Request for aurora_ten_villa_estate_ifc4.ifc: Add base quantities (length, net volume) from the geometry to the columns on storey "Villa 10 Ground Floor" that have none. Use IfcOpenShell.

First a look at what the model holds.

```python
import ifcopenshell
import ifcopenshell.util.element
import ifcopenshell.util.unit

model = ifcopenshell.open("aurora_ten_villa_estate_ifc4.ifc")
print(model.schema)
for unit_type in ("LENGTHUNIT", "AREAUNIT", "VOLUMEUNIT"):
    print(unit_type, ifcopenshell.util.unit.calculate_unit_scale(model, unit_type))
storey = next(s for s in model.by_type("IfcBuildingStorey") if s.Name == "Villa 10 Ground Floor")
columns = [e for e in ifcopenshell.util.element.get_decomposition(storey) if e.is_a("IfcColumn")]
for e in sorted(columns, key=lambda e: e.id()):
    print(e.id(), e.is_a(), e.Name, list(ifcopenshell.util.element.get_psets(e, qtos_only=True)), sep=" | ")
```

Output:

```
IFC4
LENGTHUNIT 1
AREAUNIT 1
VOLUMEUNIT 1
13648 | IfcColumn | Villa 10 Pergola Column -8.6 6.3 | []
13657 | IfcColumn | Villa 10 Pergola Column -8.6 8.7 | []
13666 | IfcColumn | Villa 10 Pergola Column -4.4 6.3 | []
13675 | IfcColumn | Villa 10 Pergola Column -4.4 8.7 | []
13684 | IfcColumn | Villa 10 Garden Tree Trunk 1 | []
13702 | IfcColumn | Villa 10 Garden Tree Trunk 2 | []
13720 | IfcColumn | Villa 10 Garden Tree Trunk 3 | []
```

```python
import ifcopenshell
import ifcopenshell.api.pset
import ifcopenshell.geom
import ifcopenshell.util.element
import ifcopenshell.util.shape
import ifcopenshell.util.unit

model = ifcopenshell.open("aurora_ten_villa_estate_ifc4.ifc")
unit_scale = ifcopenshell.util.unit.calculate_unit_scale(model)
volume_scale = ifcopenshell.util.unit.calculate_unit_scale(model, "VOLUMEUNIT")
settings = ifcopenshell.geom.settings()

storey = next(s for s in model.by_type("IfcBuildingStorey") if s.Name == "Villa 10 Ground Floor")
columns = [e for e in ifcopenshell.util.element.get_decomposition(storey) if e.is_a("IfcColumn")]

for e in sorted(columns, key=lambda e: e.id()):
    if ifcopenshell.util.element.get_psets(e, qtos_only=True, should_inherit=False):
        continue
    # Geometry comes back in metres, in the element's own axes.
    shape = ifcopenshell.geom.create_shape(settings, e)
    values = {
        "Length": ifcopenshell.util.shape.get_z(shape.geometry) / unit_scale,
        "NetVolume": ifcopenshell.util.shape.get_volume(shape.geometry) / volume_scale,
    }
    qto = ifcopenshell.api.pset.add_qto(model, product=e, name="Qto_ColumnBaseQuantities")
    ifcopenshell.api.pset.edit_qto(model, qto=qto, properties=values)
    print(e.id(), {k: round(v, 3) for k, v in values.items()})

model.write("aurora_ten_villa_estate_ifc4_v2.ifc")
```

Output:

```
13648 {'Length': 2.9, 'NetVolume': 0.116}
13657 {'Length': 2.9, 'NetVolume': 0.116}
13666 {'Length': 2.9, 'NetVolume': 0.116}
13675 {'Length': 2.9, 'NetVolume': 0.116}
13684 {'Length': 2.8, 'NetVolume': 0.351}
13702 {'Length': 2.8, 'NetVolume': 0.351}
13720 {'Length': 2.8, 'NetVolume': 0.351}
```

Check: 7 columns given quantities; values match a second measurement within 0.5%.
